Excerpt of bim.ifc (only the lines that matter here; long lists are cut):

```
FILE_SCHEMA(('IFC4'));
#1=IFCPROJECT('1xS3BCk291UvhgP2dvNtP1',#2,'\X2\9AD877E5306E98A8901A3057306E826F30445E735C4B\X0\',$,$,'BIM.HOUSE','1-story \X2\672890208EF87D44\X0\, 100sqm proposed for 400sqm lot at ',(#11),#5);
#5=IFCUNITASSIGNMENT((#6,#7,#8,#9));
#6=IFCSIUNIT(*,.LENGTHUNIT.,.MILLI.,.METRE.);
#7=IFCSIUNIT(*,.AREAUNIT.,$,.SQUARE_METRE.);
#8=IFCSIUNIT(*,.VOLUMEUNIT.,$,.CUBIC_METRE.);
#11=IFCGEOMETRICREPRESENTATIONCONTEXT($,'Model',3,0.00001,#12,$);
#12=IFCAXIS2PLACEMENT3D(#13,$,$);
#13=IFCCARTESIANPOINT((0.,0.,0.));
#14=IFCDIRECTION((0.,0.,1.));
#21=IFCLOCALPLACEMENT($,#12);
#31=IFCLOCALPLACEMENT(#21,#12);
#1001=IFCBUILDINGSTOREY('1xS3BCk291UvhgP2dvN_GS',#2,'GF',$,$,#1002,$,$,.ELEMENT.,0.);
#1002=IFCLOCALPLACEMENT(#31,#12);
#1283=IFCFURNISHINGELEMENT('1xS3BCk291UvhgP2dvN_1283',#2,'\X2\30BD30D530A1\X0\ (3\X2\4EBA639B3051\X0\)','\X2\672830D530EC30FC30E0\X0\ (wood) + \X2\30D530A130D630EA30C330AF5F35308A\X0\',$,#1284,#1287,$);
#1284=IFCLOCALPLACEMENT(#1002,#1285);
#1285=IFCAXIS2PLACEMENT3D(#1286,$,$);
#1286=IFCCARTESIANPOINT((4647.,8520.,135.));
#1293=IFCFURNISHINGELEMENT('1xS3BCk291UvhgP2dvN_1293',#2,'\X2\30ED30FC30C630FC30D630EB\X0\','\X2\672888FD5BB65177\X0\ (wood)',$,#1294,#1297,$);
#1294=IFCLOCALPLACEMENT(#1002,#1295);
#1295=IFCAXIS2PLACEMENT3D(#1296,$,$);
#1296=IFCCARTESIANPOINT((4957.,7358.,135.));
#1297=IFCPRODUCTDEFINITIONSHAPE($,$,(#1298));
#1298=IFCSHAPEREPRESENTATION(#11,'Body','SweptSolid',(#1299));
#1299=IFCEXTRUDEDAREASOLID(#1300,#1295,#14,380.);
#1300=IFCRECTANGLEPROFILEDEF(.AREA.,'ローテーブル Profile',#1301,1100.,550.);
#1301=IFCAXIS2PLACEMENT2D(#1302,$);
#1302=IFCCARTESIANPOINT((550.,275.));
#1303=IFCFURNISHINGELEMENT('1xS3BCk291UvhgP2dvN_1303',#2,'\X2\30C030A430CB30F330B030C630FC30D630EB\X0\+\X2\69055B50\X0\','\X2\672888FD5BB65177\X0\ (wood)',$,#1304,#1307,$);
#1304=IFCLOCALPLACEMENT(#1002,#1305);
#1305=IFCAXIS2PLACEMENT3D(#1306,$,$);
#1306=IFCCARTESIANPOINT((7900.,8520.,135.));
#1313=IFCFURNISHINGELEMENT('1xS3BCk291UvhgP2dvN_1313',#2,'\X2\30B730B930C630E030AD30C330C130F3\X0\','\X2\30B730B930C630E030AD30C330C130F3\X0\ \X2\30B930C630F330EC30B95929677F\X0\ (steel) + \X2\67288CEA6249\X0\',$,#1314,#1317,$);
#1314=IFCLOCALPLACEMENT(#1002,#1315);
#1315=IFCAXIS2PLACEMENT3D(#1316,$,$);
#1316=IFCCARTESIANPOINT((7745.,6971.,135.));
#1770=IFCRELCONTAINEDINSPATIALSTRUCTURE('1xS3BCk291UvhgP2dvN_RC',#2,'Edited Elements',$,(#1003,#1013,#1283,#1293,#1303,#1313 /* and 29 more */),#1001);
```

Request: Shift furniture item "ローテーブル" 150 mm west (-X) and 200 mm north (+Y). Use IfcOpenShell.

```python
import ifcopenshell
import ifcopenshell.api.geometry
import ifcopenshell.util.placement
import ifcopenshell.util.unit

model = ifcopenshell.open("bim.ifc")
unit_scale = ifcopenshell.util.unit.calculate_unit_scale(model)

item = model.by_id(1293)
matrix = ifcopenshell.util.placement.get_local_placement(item.ObjectPlacement)
matrix[0, 3] -= 0.15 / unit_scale
matrix[1, 3] += 0.2 / unit_scale
ifcopenshell.api.geometry.edit_object_placement(model, product=item, matrix=matrix, is_si=False)

print(ifcopenshell.util.placement.get_local_placement(item.ObjectPlacement).round(3) + 0.0)

model.write("bim_v2.ifc")
```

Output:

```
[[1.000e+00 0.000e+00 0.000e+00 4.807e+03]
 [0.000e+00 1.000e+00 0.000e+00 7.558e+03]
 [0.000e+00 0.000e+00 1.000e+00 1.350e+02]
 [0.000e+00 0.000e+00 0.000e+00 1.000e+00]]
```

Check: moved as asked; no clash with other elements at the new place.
